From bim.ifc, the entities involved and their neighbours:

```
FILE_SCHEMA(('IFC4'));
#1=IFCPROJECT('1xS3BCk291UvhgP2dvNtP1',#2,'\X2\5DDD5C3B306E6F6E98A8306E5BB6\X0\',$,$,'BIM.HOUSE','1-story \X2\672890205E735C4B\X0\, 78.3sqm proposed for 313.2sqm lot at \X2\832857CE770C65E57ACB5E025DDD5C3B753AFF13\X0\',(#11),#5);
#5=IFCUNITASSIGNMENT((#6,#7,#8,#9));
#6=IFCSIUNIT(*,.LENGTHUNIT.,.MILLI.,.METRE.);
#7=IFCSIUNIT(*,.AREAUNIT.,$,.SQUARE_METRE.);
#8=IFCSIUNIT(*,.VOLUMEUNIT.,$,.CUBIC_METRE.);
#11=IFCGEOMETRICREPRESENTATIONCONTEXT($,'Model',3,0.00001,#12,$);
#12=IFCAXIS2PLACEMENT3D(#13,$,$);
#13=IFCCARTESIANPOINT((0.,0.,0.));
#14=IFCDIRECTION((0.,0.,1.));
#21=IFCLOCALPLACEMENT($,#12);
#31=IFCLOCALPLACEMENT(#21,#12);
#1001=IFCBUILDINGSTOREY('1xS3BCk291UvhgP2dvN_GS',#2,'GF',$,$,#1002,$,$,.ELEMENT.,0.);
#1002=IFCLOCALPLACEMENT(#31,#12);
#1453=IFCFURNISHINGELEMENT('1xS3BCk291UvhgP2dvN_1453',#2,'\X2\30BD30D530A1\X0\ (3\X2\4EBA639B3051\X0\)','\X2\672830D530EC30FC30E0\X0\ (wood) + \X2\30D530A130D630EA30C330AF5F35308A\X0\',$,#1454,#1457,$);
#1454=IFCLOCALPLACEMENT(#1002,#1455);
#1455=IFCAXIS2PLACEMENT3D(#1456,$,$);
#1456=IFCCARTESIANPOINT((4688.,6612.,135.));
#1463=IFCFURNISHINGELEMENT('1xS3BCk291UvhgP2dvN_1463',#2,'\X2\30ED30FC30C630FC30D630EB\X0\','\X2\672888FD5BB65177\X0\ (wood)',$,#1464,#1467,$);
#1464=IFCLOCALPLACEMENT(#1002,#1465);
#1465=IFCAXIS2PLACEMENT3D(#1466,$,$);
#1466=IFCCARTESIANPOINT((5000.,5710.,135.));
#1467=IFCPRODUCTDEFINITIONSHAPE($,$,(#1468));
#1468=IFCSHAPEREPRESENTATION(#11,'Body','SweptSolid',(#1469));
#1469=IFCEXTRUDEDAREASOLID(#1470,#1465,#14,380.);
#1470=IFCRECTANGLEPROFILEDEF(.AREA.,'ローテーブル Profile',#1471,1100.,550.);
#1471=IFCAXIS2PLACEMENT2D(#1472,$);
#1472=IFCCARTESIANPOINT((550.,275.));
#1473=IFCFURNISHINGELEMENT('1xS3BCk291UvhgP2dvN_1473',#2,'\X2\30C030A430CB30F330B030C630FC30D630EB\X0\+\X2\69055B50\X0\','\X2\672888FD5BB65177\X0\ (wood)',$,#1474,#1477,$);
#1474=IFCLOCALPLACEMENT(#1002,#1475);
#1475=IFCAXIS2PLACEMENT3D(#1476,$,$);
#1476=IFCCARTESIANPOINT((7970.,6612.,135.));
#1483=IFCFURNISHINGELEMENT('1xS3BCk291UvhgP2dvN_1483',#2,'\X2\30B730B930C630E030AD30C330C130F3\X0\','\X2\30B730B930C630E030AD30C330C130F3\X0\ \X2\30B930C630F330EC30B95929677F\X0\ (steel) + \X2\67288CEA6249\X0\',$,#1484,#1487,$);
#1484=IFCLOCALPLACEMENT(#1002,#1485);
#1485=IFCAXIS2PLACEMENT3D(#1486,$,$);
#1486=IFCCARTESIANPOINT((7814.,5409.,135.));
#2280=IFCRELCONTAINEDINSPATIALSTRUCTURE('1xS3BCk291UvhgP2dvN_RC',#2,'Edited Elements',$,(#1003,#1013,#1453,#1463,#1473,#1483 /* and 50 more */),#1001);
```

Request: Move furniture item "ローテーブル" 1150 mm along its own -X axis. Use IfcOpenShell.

```python
import ifcopenshell
import ifcopenshell.api.geometry
import ifcopenshell.util.placement

model = ifcopenshell.open("bim.ifc")

item = model.by_id(1463)
matrix = ifcopenshell.util.placement.get_local_placement(item.ObjectPlacement)
matrix[:3, 3] -= matrix[:3, 0] * 1150.0
ifcopenshell.api.geometry.edit_object_placement(model, product=item, matrix=matrix, is_si=False)

print(ifcopenshell.util.placement.get_local_placement(item.ObjectPlacement).round(3) + 0.0)

model.write("bim_edited.ifc")
```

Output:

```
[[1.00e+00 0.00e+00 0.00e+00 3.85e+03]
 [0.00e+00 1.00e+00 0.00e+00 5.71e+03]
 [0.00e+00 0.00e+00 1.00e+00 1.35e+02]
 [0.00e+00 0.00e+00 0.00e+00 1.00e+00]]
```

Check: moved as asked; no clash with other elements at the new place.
